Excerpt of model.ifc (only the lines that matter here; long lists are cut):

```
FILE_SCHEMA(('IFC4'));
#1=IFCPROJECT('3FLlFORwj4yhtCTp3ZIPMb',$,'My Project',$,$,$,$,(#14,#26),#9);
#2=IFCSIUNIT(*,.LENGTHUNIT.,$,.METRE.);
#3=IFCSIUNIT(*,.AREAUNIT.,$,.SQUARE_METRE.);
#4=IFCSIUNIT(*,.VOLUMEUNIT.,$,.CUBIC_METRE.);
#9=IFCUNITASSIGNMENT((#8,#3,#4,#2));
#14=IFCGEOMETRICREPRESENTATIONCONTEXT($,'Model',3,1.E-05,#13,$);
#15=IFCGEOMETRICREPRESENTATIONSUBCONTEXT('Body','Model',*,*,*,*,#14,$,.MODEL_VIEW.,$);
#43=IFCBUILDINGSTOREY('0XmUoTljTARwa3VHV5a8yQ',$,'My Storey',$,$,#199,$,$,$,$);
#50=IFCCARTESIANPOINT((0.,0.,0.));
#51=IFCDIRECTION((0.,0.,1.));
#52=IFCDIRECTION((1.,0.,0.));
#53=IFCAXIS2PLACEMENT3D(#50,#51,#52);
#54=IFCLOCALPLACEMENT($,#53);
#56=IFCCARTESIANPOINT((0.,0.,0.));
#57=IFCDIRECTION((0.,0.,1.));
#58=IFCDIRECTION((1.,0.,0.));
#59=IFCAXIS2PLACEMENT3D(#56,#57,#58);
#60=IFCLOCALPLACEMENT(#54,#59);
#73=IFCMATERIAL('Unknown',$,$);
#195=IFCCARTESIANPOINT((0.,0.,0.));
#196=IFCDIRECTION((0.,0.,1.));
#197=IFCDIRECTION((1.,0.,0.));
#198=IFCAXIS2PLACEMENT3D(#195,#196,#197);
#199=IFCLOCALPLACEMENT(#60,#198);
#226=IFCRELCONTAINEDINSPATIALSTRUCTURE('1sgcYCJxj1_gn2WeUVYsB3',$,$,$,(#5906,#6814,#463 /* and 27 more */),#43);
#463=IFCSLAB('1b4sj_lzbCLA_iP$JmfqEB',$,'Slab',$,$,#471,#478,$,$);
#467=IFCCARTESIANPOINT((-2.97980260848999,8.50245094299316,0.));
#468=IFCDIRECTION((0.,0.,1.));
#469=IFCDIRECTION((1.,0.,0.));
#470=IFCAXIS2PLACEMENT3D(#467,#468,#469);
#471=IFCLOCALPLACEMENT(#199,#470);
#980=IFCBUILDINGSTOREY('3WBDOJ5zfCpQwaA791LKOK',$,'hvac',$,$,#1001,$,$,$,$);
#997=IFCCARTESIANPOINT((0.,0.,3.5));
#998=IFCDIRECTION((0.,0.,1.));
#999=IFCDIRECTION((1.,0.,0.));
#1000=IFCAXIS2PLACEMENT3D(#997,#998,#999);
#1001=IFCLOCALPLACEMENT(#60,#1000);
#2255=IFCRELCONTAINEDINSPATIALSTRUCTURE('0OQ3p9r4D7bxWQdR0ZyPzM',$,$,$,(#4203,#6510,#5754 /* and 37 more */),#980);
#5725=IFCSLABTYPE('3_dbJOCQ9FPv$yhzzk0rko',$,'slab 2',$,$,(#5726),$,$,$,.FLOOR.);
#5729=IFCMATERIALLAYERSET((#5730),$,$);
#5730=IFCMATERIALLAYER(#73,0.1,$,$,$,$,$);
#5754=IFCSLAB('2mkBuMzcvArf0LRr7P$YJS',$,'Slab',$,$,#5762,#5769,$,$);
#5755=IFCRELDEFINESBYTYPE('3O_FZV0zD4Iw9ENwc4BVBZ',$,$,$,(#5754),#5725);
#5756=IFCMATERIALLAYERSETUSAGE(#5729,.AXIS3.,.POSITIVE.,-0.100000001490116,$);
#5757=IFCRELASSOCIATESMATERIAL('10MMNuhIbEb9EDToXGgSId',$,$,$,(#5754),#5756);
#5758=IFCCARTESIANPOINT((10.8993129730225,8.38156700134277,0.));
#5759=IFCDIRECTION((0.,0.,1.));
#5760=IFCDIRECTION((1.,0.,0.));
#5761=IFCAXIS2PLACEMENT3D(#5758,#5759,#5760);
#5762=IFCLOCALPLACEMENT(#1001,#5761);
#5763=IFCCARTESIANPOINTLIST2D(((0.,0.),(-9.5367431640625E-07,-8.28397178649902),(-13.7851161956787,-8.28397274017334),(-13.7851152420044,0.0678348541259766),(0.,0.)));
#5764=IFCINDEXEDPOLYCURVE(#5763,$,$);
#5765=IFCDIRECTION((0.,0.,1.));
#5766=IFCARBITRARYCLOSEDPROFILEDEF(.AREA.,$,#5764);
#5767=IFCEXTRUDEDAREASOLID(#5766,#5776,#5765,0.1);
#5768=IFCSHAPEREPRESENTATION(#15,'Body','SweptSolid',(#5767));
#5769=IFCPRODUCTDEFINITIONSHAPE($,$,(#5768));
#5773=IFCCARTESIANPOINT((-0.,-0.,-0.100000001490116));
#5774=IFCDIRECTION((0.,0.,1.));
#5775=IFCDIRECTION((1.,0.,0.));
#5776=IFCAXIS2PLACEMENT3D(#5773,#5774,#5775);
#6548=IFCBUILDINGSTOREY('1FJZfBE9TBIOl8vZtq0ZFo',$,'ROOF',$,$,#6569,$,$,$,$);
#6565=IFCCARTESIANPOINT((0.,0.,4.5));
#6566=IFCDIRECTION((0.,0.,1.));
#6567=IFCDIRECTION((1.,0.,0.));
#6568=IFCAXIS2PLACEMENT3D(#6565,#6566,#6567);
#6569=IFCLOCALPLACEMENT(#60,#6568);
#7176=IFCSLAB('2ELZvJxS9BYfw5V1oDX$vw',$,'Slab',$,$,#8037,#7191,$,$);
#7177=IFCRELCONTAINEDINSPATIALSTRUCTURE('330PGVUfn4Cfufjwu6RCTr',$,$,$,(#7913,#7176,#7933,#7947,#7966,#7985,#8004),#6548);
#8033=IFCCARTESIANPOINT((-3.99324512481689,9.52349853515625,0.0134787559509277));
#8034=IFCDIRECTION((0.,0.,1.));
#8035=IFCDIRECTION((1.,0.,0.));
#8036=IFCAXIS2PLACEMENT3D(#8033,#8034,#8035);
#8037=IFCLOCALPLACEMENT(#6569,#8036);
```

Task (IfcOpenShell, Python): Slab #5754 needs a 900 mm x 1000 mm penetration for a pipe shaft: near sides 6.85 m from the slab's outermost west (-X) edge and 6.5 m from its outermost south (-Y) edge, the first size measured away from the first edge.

```python
import numpy as np
import ifcopenshell
import ifcopenshell.api.feature
import ifcopenshell.api.geometry
import ifcopenshell.api.root
import ifcopenshell.geom
import ifcopenshell.util.placement
import ifcopenshell.util.representation
import ifcopenshell.util.shape
import ifcopenshell.util.unit

model = ifcopenshell.open("model.ifc")
unit_scale = ifcopenshell.util.unit.calculate_unit_scale(model)
settings = ifcopenshell.geom.settings()


def volume(element):
    """Net volume in cubic metres, openings subtracted."""
    shape = ifcopenshell.geom.create_shape(settings, element)
    return ifcopenshell.util.shape.get_volume(shape.geometry)


slab = model.by_id(5754)
before = volume(slab)

# Extent in the slab's own axes, in metres. The edges named are its -X and -Y sides.
slab_shape = ifcopenshell.geom.create_shape(settings, slab)
vertices = ifcopenshell.util.shape.get_vertices(slab_shape.geometry)
x_min, y_min, bottom = vertices.min(axis=0)
top = vertices[:, 2].max()

opening = ifcopenshell.api.root.create_entity(model, ifc_class="IfcOpeningElement", name="Pipe shaft opening", predefined_type="OPENING")
context = ifcopenshell.util.representation.get_context(model, "Model", "Body", "MODEL_VIEW")
width, depth = 0.9, 1
outline = [(0.0, 0.0), (width, 0.0), (width, depth), (0.0, depth), (0.0, 0.0)]
# Overshoot both faces by 50 mm so the cut is clean.
shape = ifcopenshell.api.geometry.add_slab_representation(
    model, context=context, depth=top - bottom + 0.1, polyline=outline
)
ifcopenshell.api.geometry.assign_representation(model, product=opening, representation=shape)

matrix = ifcopenshell.util.placement.get_local_placement(slab.ObjectPlacement)
matrix[:, 3] = matrix @ np.append(np.array([x_min + 6.85, y_min + 6.5, bottom - 0.05]) / unit_scale, 1.0)
ifcopenshell.api.geometry.edit_object_placement(model, product=opening, matrix=matrix, is_si=False)
ifcopenshell.api.feature.add_feature(model, feature=opening, element=slab)

after = volume(slab)

print(f"slab volume {before:.3f} -> {after:.3f} m3")

model.write("model_v2.ifc")
```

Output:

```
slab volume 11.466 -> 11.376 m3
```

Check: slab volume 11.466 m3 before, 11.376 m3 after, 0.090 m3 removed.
